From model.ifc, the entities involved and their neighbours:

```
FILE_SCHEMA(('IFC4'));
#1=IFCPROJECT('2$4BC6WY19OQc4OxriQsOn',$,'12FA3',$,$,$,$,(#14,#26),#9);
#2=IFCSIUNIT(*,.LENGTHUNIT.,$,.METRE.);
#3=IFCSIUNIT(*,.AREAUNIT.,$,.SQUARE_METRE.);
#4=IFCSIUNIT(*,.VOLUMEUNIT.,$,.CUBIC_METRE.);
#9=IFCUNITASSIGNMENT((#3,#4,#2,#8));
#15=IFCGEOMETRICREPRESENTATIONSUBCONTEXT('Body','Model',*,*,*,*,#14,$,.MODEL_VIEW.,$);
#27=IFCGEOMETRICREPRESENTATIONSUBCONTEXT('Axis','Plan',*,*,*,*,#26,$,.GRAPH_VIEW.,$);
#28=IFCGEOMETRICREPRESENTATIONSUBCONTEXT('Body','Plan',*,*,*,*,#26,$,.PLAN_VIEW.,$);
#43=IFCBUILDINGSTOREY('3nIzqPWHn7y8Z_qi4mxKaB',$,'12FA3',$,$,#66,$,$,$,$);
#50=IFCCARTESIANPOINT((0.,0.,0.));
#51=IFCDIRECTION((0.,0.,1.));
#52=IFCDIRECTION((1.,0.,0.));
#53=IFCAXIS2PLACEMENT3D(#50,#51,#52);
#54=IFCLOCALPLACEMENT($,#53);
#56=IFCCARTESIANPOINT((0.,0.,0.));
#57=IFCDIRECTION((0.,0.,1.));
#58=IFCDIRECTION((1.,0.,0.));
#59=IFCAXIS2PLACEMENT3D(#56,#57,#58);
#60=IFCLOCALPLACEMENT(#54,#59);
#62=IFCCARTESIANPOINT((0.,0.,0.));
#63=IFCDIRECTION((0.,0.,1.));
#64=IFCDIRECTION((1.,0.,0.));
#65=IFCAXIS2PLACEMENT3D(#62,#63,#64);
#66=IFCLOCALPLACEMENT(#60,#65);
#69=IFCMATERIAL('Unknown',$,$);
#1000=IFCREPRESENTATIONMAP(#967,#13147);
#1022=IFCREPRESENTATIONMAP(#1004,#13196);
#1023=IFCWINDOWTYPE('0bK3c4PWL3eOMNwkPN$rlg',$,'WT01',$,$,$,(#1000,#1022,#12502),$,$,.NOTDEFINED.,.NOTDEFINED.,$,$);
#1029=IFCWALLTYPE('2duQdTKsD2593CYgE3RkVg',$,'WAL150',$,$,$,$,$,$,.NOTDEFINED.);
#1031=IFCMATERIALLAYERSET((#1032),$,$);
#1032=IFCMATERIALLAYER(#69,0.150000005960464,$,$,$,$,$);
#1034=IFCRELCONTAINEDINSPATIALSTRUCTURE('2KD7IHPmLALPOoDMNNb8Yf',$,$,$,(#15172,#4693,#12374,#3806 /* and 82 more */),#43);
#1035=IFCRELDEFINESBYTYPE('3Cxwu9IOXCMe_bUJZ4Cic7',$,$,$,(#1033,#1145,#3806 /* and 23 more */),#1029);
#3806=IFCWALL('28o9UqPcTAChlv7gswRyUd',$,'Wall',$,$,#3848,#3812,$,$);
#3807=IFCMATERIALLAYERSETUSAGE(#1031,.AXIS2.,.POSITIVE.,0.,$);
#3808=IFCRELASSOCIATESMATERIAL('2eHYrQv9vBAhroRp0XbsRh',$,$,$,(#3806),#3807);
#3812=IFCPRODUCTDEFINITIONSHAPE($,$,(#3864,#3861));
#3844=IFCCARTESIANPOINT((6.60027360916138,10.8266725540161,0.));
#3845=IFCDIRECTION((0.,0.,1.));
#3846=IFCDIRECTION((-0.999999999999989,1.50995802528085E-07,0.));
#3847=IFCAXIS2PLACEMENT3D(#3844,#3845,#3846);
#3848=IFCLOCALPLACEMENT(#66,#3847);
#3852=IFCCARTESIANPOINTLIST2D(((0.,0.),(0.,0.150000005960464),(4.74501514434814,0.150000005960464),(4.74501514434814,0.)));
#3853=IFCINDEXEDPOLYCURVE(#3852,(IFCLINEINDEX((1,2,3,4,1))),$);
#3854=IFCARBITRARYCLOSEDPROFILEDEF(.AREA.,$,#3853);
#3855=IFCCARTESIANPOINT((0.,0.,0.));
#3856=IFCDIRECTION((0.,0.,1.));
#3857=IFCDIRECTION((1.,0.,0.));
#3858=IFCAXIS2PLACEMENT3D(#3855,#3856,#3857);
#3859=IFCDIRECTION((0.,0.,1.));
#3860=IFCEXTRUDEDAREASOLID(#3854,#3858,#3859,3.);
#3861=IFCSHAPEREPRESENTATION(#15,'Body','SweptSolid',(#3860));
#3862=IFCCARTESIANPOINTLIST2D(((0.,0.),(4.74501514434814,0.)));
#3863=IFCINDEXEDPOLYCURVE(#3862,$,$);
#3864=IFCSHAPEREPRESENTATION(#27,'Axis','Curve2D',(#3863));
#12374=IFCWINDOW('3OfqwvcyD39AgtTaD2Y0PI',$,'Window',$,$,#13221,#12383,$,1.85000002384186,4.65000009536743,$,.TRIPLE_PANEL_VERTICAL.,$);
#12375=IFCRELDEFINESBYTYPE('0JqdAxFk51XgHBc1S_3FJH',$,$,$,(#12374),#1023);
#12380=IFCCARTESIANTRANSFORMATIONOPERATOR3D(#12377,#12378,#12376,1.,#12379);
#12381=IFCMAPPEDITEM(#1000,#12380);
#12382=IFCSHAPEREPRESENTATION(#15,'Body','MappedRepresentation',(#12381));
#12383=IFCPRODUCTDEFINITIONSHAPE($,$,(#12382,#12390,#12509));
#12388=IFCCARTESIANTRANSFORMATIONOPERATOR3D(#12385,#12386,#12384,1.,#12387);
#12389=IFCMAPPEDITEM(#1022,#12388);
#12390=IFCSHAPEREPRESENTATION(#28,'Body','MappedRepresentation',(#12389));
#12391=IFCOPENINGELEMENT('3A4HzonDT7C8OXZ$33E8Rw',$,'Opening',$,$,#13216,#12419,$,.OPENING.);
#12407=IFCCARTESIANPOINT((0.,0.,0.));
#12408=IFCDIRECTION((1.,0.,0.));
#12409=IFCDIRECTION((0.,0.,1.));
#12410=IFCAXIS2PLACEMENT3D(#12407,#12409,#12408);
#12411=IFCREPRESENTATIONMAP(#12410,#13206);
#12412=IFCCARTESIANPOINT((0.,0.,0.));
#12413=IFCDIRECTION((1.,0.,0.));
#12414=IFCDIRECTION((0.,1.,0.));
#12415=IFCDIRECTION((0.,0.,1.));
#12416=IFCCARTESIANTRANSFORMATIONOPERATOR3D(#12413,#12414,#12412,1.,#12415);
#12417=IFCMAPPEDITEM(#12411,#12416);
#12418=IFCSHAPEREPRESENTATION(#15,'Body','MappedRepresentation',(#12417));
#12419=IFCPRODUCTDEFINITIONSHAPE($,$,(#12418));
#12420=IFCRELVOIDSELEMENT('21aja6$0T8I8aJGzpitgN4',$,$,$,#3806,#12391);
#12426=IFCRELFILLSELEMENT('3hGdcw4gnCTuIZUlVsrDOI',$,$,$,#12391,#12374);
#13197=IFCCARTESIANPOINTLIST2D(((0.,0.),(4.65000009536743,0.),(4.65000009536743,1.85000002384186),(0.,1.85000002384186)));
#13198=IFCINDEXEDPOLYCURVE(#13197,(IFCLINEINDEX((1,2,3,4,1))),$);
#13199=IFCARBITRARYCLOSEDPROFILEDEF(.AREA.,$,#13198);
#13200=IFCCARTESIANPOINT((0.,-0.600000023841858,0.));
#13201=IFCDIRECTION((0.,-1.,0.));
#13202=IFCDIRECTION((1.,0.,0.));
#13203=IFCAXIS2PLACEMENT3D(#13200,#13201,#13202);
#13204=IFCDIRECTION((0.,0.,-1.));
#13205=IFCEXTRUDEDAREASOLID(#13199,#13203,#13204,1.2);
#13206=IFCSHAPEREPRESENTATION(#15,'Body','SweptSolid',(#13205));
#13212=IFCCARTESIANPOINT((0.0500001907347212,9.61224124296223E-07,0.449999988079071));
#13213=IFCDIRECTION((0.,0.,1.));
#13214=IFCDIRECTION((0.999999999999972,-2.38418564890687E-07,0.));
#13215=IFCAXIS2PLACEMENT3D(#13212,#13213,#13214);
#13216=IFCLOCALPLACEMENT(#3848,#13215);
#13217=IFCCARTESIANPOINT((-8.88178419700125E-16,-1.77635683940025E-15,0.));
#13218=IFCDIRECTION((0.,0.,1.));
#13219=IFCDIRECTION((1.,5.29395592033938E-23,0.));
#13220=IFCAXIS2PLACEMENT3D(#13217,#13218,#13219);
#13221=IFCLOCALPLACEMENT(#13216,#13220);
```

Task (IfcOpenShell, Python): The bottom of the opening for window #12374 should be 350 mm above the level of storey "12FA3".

```python
import numpy as np
import ifcopenshell
import ifcopenshell.api.geometry
import ifcopenshell.geom
import ifcopenshell.util.element
import ifcopenshell.util.placement
import ifcopenshell.util.shape
import ifcopenshell.util.unit

model = ifcopenshell.open("model.ifc")
unit_scale = ifcopenshell.util.unit.calculate_unit_scale(model)

window = model.by_guid("3OfqwvcyD39AgtTaD2Y0PI")
opening = window.FillsVoids[0].RelatingOpeningElement
storey = ifcopenshell.util.element.get_container(window, ifc_class="IfcBuildingStorey")
level = ifcopenshell.util.placement.get_local_placement(storey.ObjectPlacement)[2, 3]

# The opening's origin need not be at the sill, so measure its lowest point.
shape = ifcopenshell.geom.create_shape(ifcopenshell.geom.settings(), opening)
bottom = ifcopenshell.util.shape.get_shape_bottom_elevation(shape, shape.geometry) / unit_scale
dz = level + 0.35 / unit_scale - bottom

shift = np.array([0.0, 0.0, dz])
# The window is placed relative to its opening, so it follows when the opening moves.
matrix = ifcopenshell.util.placement.get_local_placement(opening.ObjectPlacement)
matrix[:3, 3] += shift
ifcopenshell.api.geometry.edit_object_placement(
    model, product=opening, matrix=matrix, is_si=False, should_transform_children=True
)

print(f"moved by {dz * unit_scale:+.3f} m")

model.write("model_v2.ifc")
```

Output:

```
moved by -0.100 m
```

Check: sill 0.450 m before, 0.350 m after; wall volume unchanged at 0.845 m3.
